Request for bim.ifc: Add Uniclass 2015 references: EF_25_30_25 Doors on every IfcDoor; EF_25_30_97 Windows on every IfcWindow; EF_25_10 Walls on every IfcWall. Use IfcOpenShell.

First a look at what the model holds.

```python
import ifcopenshell

model = ifcopenshell.open("bim.ifc")
print(model.schema)
print("classifications:", [c.Name for c in model.by_type("IfcClassification")])
for ifc_class in ("IfcDoor", "IfcRoof", "IfcStair", "IfcWall", "IfcWindow"):
    print(ifc_class, len(model.by_type(ifc_class)))
```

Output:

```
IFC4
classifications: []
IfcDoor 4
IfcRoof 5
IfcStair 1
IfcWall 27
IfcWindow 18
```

```python
import ifcopenshell
import ifcopenshell.api.classification

model = ifcopenshell.open("bim.ifc")

system = ifcopenshell.api.classification.add_classification(model, classification="Uniclass 2015")

codes = {
    "IfcDoor": ("EF_25_30_25", "Doors"),
    "IfcWindow": ("EF_25_30_97", "Windows"),
    "IfcWall": ("EF_25_10", "Walls"),
}
for ifc_class, (code, name) in codes.items():
    products = model.by_type(ifc_class)
    ifcopenshell.api.classification.add_reference(
        model, products=products, classification=system, identification=code, name=name
    )
    print(code, len(products))

model.write("bim_edited.ifc")
```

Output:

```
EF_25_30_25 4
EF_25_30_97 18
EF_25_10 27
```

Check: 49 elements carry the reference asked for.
